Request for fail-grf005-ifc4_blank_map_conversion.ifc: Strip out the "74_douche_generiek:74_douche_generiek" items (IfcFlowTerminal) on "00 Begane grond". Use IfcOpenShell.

First a look at what the model holds.

```python
import ifcopenshell
import ifcopenshell.util.element

model = ifcopenshell.open("fail-grf005-ifc4_blank_map_conversion.ifc")
print(model.schema)
storey = next(s for s in model.by_type("IfcBuildingStorey") if s.Name == "00 Begane grond")
terminals = [e for e in ifcopenshell.util.element.get_decomposition(storey) if e.is_a("IfcFlowTerminal")]
seen = {}
for e in terminals:
    element_type = ifcopenshell.util.element.get_type(e)
    name = element_type.Name if element_type not in (None, e) else None
    seen[name] = seen.get(name, 0) + 1
for name, count in sorted(seen.items(), key=str):
    print(count, "x", name)
```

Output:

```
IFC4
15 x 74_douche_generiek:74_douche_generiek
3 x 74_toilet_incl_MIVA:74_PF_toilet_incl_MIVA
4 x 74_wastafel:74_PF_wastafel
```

```python
import ifcopenshell
import ifcopenshell.api.root
import ifcopenshell.util.element

model = ifcopenshell.open("fail-grf005-ifc4_blank_map_conversion.ifc")

storey = next(s for s in model.by_type("IfcBuildingStorey") if s.Name == "00 Begane grond")
terminals = [e for e in ifcopenshell.util.element.get_decomposition(storey) if e.is_a("IfcFlowTerminal")]
targets = [e for e in terminals if (t := ifcopenshell.util.element.get_type(e)) not in (None, e) and t.Name == "74_douche_generiek:74_douche_generiek"]

for e in targets:
    ifcopenshell.api.root.remove_product(model, product=e)
print(len(targets), "removed")

model.write("fail-grf005-ifc4_blank_map_conversion_edited.ifc")
```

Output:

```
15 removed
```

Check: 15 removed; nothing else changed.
